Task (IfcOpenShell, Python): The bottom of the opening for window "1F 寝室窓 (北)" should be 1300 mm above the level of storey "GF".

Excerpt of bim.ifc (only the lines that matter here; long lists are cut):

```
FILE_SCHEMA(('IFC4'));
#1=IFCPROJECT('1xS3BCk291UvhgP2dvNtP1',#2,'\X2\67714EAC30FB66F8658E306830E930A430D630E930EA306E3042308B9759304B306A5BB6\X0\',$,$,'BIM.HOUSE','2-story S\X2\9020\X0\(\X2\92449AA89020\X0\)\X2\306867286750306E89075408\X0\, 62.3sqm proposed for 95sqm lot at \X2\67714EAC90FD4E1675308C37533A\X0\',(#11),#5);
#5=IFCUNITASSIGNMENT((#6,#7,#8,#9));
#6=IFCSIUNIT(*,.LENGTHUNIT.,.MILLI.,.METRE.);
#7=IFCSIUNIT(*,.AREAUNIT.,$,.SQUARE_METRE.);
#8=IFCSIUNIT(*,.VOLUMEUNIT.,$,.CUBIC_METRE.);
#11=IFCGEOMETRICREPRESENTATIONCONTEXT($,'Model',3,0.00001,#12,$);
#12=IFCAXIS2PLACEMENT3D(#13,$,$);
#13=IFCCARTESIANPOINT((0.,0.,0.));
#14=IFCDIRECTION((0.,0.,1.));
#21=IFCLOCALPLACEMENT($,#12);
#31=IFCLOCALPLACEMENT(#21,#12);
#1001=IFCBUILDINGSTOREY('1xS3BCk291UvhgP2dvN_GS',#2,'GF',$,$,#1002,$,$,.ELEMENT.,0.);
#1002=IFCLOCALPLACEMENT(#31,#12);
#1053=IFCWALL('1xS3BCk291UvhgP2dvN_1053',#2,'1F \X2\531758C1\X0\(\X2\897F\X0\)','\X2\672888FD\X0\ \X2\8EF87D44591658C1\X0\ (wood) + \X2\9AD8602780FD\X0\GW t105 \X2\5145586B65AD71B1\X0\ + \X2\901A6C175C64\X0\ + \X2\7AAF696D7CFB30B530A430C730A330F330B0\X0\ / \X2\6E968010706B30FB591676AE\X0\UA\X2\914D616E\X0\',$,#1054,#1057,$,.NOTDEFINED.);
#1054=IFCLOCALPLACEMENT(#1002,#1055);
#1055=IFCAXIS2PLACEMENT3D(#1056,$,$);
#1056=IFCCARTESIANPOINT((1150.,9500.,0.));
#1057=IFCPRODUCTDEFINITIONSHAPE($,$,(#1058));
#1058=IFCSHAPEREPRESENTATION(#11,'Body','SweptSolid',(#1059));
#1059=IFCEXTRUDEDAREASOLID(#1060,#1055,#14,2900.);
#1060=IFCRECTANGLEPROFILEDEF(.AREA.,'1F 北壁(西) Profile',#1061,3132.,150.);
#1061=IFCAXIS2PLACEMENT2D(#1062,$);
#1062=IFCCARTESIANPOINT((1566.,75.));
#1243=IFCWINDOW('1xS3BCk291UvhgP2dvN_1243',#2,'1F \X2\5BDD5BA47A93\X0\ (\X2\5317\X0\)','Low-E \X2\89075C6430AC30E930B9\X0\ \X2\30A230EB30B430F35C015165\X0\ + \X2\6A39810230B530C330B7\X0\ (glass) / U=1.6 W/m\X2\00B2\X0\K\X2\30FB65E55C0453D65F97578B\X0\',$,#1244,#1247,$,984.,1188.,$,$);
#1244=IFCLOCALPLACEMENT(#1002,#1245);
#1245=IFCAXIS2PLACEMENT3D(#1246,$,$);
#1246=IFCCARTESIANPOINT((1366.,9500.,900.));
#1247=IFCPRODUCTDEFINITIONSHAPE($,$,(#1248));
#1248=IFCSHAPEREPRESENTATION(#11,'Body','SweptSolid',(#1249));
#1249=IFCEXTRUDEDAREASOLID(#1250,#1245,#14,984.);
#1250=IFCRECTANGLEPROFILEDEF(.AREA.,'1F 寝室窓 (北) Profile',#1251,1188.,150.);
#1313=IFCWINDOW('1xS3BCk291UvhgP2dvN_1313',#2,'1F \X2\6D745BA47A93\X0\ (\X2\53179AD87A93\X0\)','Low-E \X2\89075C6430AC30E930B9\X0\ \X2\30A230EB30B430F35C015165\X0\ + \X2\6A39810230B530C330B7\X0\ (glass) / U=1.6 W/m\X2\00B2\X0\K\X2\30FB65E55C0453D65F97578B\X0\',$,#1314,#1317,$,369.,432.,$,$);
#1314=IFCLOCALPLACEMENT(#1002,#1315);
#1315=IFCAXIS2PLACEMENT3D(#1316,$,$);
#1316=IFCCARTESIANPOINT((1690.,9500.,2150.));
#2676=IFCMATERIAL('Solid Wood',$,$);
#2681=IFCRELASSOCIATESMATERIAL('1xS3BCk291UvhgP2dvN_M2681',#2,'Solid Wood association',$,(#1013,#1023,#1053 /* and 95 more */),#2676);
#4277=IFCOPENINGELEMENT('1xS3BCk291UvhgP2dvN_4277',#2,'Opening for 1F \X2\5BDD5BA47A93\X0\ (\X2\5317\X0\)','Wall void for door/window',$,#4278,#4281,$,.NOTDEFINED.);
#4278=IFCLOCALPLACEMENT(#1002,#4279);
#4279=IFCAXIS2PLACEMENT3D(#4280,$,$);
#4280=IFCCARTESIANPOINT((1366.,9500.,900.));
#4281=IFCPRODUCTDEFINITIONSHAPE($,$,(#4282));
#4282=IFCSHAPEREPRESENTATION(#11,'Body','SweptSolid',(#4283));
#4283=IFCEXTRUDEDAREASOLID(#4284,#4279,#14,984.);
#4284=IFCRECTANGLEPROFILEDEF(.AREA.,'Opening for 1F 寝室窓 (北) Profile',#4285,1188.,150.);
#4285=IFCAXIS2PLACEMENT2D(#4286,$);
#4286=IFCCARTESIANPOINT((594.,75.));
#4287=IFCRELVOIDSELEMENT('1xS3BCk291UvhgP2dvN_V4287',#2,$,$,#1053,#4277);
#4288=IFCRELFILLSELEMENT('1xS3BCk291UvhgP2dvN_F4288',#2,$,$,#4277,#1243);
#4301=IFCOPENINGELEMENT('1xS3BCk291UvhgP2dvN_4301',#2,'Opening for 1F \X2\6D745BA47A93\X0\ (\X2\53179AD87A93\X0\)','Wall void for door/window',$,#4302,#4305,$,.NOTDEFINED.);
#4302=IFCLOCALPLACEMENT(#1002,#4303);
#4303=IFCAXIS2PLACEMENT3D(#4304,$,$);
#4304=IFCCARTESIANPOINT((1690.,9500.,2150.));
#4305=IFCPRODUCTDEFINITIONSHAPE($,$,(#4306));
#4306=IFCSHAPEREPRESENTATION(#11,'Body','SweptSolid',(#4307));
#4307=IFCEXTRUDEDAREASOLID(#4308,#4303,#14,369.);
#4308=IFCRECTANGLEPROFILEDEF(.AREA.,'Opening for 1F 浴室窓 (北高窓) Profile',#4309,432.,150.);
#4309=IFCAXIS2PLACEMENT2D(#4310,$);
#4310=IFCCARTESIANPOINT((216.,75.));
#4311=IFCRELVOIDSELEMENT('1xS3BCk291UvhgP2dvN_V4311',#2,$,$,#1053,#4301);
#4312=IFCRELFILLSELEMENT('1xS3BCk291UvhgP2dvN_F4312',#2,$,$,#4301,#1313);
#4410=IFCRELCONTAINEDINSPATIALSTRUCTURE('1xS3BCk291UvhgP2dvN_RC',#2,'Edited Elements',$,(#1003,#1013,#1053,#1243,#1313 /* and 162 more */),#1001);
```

```python
import numpy as np
import ifcopenshell
import ifcopenshell.api.geometry
import ifcopenshell.geom
import ifcopenshell.util.element
import ifcopenshell.util.placement
import ifcopenshell.util.shape
import ifcopenshell.util.unit

model = ifcopenshell.open("bim.ifc")
unit_scale = ifcopenshell.util.unit.calculate_unit_scale(model)

window = model.by_guid("1xS3BCk291UvhgP2dvN_1243")
opening = window.FillsVoids[0].RelatingOpeningElement
storey = ifcopenshell.util.element.get_container(window, ifc_class="IfcBuildingStorey")
level = ifcopenshell.util.placement.get_local_placement(storey.ObjectPlacement)[2, 3]

# The opening's origin need not be at the sill, so measure its lowest point.
shape = ifcopenshell.geom.create_shape(ifcopenshell.geom.settings(), opening)
bottom = ifcopenshell.util.shape.get_shape_bottom_elevation(shape, shape.geometry) / unit_scale
dz = level + 1.3 / unit_scale - bottom

shift = np.array([0.0, 0.0, dz])
# The window is not placed relative to its opening, so move both.
for product in (opening, window):
    matrix = ifcopenshell.util.placement.get_local_placement(product.ObjectPlacement)
    matrix[:3, 3] += shift
    ifcopenshell.api.geometry.edit_object_placement(model, product=product, matrix=matrix, is_si=False)

print(f"moved by {dz * unit_scale:+.3f} m")

model.write("bim_updated.ifc")
```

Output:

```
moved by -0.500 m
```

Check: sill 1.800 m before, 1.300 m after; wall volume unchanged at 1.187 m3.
